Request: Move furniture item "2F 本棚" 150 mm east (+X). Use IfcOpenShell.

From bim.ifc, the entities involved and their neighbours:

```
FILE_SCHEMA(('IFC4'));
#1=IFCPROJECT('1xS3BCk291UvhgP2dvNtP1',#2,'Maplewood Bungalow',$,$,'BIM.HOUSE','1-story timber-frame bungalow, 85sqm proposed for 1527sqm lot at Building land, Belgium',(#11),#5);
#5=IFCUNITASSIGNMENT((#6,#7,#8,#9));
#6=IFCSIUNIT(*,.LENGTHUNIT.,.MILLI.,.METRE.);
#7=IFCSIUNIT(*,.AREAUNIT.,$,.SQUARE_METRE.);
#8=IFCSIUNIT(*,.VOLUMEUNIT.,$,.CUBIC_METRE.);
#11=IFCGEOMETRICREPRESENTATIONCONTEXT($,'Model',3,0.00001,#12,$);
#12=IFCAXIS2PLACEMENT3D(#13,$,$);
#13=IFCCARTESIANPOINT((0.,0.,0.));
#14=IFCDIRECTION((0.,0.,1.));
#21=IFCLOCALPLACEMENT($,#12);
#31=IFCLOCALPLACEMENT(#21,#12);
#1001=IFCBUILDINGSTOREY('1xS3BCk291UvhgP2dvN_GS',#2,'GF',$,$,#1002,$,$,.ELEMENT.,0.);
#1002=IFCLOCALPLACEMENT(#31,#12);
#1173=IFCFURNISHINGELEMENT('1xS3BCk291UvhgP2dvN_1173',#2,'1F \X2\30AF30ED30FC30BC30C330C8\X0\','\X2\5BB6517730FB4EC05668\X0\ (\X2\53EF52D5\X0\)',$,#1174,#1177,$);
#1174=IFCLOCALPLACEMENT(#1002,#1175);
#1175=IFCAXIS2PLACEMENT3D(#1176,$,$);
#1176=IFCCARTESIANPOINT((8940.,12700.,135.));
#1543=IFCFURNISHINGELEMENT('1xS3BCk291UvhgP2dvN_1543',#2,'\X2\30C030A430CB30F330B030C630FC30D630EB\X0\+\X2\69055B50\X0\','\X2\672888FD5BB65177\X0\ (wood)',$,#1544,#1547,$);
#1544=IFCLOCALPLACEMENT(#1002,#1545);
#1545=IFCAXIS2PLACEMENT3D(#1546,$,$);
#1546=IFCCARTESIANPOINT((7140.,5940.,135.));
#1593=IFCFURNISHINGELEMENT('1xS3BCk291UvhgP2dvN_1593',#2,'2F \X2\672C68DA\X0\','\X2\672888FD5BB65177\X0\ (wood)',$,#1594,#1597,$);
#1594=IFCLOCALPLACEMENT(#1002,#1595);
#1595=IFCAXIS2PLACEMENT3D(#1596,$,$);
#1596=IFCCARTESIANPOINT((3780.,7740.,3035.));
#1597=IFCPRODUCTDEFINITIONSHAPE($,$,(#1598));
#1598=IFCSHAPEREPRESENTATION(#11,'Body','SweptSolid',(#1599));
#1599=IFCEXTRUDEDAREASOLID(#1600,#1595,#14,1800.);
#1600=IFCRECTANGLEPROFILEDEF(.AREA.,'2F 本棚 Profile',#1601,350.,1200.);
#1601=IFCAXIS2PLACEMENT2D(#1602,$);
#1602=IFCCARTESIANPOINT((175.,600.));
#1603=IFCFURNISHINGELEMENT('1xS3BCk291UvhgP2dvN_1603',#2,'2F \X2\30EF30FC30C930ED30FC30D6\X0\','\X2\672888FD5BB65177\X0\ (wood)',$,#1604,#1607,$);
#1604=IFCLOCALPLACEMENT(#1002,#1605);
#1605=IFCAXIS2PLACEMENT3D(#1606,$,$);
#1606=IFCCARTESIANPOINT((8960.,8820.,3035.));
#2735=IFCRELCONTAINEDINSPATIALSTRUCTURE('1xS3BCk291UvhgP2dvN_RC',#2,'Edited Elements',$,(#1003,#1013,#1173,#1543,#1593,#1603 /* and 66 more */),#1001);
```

```python
import ifcopenshell
import ifcopenshell.api.geometry
import ifcopenshell.util.placement
import ifcopenshell.util.unit

model = ifcopenshell.open("bim.ifc")
unit_scale = ifcopenshell.util.unit.calculate_unit_scale(model)

item = model.by_guid("1xS3BCk291UvhgP2dvN_1593")
matrix = ifcopenshell.util.placement.get_local_placement(item.ObjectPlacement)
matrix[0, 3] += 0.15 / unit_scale
ifcopenshell.api.geometry.edit_object_placement(model, product=item, matrix=matrix, is_si=False)

print(ifcopenshell.util.placement.get_local_placement(item.ObjectPlacement).round(3) + 0.0)

model.write("bim_rev.ifc")
```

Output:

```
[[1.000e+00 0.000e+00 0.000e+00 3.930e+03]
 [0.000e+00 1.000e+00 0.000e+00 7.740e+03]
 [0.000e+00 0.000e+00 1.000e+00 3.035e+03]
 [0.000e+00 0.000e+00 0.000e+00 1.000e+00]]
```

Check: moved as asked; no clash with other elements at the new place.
